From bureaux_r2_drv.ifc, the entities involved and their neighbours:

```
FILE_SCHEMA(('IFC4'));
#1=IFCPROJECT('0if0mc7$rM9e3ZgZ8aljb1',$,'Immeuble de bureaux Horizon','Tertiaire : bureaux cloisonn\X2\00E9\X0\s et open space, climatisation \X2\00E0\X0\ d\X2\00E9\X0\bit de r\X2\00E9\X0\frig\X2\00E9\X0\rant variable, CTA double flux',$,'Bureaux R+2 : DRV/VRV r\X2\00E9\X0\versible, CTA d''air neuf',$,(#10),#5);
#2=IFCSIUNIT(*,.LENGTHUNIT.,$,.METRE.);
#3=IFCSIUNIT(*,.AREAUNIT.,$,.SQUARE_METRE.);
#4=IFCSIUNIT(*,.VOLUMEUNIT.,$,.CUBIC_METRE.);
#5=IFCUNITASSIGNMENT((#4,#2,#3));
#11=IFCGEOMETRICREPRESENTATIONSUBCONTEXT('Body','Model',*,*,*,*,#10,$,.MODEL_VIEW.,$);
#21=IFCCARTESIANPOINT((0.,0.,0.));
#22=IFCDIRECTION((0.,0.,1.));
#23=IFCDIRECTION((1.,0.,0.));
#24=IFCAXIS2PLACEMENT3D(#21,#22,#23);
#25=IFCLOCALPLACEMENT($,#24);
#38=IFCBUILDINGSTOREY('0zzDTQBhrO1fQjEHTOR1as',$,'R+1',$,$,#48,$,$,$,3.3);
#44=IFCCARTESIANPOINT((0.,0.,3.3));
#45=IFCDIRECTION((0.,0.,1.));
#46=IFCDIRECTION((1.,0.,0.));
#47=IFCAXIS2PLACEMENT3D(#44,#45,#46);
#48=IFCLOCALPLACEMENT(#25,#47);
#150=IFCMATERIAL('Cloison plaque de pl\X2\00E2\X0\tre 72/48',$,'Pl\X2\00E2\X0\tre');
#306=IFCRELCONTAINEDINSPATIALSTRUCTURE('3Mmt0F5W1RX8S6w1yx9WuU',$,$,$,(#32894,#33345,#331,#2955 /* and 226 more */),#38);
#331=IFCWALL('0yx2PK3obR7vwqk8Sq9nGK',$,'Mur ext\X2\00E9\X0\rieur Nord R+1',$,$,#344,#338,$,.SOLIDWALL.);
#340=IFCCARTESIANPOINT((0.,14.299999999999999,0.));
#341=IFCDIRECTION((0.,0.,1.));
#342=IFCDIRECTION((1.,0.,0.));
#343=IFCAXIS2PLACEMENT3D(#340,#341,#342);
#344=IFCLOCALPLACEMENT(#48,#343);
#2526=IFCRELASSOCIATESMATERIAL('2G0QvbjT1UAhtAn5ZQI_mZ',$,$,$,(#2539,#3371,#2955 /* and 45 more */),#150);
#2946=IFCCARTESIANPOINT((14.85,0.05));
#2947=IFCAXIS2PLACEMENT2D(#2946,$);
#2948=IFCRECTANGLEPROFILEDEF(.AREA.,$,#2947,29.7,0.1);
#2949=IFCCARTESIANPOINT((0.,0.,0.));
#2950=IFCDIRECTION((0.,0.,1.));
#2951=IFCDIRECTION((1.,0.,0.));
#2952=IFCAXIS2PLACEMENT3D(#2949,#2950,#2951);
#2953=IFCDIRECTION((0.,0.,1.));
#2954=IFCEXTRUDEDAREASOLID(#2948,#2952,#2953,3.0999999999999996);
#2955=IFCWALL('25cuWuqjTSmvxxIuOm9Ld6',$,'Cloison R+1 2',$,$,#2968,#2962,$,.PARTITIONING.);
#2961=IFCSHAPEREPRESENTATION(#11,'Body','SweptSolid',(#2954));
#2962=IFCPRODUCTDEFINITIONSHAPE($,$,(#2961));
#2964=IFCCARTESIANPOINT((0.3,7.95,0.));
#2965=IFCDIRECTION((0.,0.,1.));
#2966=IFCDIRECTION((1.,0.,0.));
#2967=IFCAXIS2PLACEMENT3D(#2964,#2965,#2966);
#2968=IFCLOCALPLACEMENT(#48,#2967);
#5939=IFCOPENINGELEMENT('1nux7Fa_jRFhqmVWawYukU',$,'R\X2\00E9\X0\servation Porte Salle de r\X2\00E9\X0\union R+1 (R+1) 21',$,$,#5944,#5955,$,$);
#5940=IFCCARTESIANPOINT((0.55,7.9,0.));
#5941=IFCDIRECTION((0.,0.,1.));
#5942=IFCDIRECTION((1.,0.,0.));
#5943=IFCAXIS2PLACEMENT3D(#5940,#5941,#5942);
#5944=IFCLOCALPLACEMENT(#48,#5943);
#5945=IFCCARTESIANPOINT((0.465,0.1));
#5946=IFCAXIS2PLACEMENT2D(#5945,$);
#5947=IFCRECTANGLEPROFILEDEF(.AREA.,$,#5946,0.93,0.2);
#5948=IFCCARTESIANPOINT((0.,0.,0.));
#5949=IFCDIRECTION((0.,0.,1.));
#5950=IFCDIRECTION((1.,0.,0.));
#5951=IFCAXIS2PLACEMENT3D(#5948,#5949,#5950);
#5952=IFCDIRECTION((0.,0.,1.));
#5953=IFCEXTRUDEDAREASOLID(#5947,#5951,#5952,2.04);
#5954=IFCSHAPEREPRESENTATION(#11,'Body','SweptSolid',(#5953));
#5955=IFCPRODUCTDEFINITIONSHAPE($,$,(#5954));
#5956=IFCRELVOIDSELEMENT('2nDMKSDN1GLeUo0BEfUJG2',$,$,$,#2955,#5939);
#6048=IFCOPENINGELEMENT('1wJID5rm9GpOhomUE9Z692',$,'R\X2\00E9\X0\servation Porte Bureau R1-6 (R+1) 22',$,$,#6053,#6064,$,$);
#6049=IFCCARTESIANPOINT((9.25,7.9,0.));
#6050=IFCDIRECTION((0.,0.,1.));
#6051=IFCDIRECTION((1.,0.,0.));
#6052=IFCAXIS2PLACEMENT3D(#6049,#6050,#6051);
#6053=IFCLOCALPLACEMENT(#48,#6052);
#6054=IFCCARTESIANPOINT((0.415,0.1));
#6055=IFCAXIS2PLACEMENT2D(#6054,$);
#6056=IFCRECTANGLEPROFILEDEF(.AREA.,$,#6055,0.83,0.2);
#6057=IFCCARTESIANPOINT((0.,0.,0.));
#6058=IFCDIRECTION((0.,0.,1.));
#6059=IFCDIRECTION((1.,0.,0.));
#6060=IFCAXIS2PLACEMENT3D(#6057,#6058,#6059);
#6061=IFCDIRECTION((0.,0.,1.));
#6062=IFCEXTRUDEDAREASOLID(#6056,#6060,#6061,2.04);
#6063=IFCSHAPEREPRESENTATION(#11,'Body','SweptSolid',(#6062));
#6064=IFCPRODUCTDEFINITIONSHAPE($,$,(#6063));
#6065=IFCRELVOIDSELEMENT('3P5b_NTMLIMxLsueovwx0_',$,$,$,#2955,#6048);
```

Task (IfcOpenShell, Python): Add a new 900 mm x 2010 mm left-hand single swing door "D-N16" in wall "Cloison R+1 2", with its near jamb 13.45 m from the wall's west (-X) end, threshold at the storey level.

```python
import numpy as np
import ifcopenshell
import ifcopenshell.api.feature
import ifcopenshell.api.geometry
import ifcopenshell.api.root
import ifcopenshell.api.spatial
import ifcopenshell.geom
import ifcopenshell.util.element
import ifcopenshell.util.placement
import ifcopenshell.util.representation
import ifcopenshell.util.shape
import ifcopenshell.util.unit

model = ifcopenshell.open("bureaux_r2_drv.ifc")
unit_scale = ifcopenshell.util.unit.calculate_unit_scale(model)
settings = ifcopenshell.geom.settings()


def volume(element):
    """Net volume in cubic metres, openings subtracted."""
    shape = ifcopenshell.geom.create_shape(settings, element)
    return ifcopenshell.util.shape.get_volume(shape.geometry)


wall = model.by_id(2955)
storey = ifcopenshell.util.element.get_container(wall, ifc_class="IfcBuildingStorey")
context = ifcopenshell.util.representation.get_context(model, "Model", "Body", "MODEL_VIEW")
before = volume(wall)

width, height, from_end, sill = 0.9, 2.01, 13.45, 0.0  # metres

# The wall runs along its own X axis, and the end named is its -X end.
wall_shape = ifcopenshell.geom.create_shape(settings, wall)
x, y, z = ifcopenshell.util.shape.get_vertices(wall_shape.geometry).T
start = x.min() + from_end
face, thickness = float(y.min()), float(y.max() - y.min())
wall_matrix = ifcopenshell.util.placement.get_local_placement(wall.ObjectPlacement)
level = ifcopenshell.util.placement.get_local_placement(storey.ObjectPlacement)[2, 3]


def in_wall(x, y):
    """Placement at x, y metres in the wall's axes, at sill height."""
    matrix = wall_matrix.copy()
    matrix[:, 3] = wall_matrix @ np.array([x / unit_scale, y / unit_scale, 0.0, 1.0])
    matrix[2, 3] = level + sill / unit_scale
    return matrix


# Opening: a box that overshoots both wall faces by 50 mm.
opening = ifcopenshell.api.root.create_entity(model, ifc_class="IfcOpeningElement", predefined_type="OPENING")
box = ifcopenshell.api.geometry.add_wall_representation(
    model, context=context, length=width, height=height, thickness=thickness + 0.1
)
ifcopenshell.api.geometry.assign_representation(model, product=opening, representation=box)
ifcopenshell.api.geometry.edit_object_placement(model, product=opening, matrix=in_wall(start, face - 0.05), is_si=False)
ifcopenshell.api.feature.add_feature(model, feature=opening, element=wall)

door = ifcopenshell.api.root.create_entity(model, ifc_class="IfcDoor", name="D-N16", predefined_type="DOOR")
door.OverallWidth, door.OverallHeight = width / unit_scale, height / unit_scale
door.OperationType = "SINGLE_SWING_LEFT"
body = ifcopenshell.api.geometry.add_door_representation(
    model,
    context=context,
    overall_width=door.OverallWidth,
    overall_height=door.OverallHeight,
    operation_type="SINGLE_SWING_LEFT",
    lining_properties={"LiningDepth": thickness / unit_scale, "ThresholdDepth": thickness / unit_scale},
)
ifcopenshell.api.geometry.assign_representation(model, product=door, representation=body)
ifcopenshell.api.spatial.assign_container(model, products=[door], relating_structure=storey)
ifcopenshell.api.feature.add_filling(model, opening=opening, element=door)

# The lining spans the wall, so the door starts at the wall face.
ifcopenshell.api.geometry.edit_object_placement(model, product=door, matrix=in_wall(start, face), is_si=False)

after = volume(wall)

print(f"wall volume {before:.3f} -> {after:.3f} m3")

model.write("bureaux_r2_drv_updated.ifc")
```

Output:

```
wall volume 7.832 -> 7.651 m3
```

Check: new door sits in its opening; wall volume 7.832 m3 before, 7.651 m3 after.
